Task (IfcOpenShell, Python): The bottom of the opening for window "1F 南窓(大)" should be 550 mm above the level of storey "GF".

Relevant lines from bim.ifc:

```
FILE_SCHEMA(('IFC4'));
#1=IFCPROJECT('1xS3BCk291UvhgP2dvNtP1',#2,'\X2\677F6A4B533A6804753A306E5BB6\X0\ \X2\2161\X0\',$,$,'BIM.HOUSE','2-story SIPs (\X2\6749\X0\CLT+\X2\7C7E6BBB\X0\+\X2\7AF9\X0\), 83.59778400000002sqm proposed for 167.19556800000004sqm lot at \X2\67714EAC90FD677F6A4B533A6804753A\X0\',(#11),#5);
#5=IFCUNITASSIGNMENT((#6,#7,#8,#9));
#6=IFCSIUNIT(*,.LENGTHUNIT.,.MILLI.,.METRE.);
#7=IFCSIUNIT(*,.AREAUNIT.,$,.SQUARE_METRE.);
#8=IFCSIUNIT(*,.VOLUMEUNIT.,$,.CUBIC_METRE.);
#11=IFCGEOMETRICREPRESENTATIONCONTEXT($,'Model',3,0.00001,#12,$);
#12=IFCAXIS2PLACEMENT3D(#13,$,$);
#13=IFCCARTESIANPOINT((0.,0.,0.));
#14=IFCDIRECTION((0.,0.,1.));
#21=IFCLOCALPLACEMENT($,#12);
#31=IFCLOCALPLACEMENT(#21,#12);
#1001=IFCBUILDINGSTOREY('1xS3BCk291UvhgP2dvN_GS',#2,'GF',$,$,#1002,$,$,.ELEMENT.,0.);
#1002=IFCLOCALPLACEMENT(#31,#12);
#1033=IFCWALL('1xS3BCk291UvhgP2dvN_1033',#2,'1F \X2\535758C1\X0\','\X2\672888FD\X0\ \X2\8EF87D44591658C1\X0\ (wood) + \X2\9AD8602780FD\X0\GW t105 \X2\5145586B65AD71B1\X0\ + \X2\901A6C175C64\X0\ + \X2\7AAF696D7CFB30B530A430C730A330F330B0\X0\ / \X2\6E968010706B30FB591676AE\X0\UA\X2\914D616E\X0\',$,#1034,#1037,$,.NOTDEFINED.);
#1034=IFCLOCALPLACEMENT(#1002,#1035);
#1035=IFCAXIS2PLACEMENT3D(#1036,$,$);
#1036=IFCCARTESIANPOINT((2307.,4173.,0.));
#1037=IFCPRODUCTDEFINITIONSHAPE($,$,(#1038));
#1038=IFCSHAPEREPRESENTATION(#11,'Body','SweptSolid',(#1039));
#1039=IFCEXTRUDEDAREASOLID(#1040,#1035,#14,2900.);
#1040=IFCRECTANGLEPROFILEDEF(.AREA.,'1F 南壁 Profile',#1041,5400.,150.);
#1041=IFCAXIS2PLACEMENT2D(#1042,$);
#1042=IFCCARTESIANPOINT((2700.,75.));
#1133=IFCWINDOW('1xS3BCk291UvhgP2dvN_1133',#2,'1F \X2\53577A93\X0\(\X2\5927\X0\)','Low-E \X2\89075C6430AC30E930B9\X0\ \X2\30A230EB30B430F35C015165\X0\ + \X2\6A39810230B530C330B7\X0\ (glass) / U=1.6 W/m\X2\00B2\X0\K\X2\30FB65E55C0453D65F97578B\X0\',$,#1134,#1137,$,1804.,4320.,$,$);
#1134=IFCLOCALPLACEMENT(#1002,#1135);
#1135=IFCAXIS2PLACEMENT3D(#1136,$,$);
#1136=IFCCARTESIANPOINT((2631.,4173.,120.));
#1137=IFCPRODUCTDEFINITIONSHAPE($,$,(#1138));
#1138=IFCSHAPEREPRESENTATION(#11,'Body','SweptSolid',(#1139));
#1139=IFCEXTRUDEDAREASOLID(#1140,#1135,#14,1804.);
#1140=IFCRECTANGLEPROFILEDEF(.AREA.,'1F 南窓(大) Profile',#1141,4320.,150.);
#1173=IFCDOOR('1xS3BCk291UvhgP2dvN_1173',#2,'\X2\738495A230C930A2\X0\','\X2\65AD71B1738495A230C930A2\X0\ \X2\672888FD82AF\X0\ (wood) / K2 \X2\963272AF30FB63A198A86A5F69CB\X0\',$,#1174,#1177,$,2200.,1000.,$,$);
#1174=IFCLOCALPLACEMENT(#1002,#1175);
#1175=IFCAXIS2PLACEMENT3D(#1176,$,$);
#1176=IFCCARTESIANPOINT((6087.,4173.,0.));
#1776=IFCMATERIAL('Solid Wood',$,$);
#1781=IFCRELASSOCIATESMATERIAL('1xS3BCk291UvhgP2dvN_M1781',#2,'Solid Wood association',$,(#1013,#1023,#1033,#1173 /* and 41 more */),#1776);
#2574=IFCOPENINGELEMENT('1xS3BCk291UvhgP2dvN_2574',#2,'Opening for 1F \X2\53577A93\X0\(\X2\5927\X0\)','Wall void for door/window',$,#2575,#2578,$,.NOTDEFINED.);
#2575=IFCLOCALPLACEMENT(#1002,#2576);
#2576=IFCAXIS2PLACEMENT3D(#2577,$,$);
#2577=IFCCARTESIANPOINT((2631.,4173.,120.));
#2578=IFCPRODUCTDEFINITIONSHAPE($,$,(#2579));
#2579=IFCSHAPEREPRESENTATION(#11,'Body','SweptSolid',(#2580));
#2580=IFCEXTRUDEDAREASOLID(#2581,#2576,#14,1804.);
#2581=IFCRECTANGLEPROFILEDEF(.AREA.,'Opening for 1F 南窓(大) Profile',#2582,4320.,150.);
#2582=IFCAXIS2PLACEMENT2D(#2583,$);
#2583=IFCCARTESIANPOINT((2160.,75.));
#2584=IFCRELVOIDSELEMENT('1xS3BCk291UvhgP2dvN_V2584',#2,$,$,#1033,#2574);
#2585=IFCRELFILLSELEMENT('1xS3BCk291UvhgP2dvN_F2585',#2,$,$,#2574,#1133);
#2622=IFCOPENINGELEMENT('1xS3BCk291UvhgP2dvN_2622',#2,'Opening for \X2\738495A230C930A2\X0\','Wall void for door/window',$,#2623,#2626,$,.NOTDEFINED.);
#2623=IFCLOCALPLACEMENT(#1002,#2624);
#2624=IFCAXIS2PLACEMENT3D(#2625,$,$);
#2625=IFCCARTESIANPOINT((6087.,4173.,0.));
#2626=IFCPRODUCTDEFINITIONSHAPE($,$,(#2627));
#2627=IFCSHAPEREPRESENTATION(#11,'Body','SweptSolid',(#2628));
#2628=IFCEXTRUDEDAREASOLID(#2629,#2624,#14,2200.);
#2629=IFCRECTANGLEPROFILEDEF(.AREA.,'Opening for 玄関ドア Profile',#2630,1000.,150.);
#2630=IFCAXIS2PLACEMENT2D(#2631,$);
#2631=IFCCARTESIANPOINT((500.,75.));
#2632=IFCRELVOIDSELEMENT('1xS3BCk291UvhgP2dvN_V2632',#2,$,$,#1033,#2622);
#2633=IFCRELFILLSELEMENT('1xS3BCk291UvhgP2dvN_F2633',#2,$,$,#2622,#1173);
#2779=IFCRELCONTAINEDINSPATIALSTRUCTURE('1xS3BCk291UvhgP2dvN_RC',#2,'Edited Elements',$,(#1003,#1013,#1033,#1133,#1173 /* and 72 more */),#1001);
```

```python
import numpy as np
import ifcopenshell
import ifcopenshell.api.geometry
import ifcopenshell.geom
import ifcopenshell.util.element
import ifcopenshell.util.placement
import ifcopenshell.util.shape
import ifcopenshell.util.unit

model = ifcopenshell.open("bim.ifc")
unit_scale = ifcopenshell.util.unit.calculate_unit_scale(model)

window = model.by_guid("1xS3BCk291UvhgP2dvN_1133")
opening = window.FillsVoids[0].RelatingOpeningElement
storey = ifcopenshell.util.element.get_container(window, ifc_class="IfcBuildingStorey")
level = ifcopenshell.util.placement.get_local_placement(storey.ObjectPlacement)[2, 3]

# The opening's origin need not be at the sill, so measure its lowest point.
shape = ifcopenshell.geom.create_shape(ifcopenshell.geom.settings(), opening)
bottom = ifcopenshell.util.shape.get_shape_bottom_elevation(shape, shape.geometry) / unit_scale
dz = level + 550.0 - bottom

shift = np.array([0.0, 0.0, dz])
# The window is not placed relative to its opening, so move both.
for product in (opening, window):
    matrix = ifcopenshell.util.placement.get_local_placement(product.ObjectPlacement)
    matrix[:3, 3] += shift
    ifcopenshell.api.geometry.edit_object_placement(model, product=product, matrix=matrix, is_si=False)

print(f"moved by {dz * unit_scale:+.3f} m")

model.write("bim_edited.ifc")
```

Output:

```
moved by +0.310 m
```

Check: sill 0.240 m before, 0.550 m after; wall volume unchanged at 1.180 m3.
